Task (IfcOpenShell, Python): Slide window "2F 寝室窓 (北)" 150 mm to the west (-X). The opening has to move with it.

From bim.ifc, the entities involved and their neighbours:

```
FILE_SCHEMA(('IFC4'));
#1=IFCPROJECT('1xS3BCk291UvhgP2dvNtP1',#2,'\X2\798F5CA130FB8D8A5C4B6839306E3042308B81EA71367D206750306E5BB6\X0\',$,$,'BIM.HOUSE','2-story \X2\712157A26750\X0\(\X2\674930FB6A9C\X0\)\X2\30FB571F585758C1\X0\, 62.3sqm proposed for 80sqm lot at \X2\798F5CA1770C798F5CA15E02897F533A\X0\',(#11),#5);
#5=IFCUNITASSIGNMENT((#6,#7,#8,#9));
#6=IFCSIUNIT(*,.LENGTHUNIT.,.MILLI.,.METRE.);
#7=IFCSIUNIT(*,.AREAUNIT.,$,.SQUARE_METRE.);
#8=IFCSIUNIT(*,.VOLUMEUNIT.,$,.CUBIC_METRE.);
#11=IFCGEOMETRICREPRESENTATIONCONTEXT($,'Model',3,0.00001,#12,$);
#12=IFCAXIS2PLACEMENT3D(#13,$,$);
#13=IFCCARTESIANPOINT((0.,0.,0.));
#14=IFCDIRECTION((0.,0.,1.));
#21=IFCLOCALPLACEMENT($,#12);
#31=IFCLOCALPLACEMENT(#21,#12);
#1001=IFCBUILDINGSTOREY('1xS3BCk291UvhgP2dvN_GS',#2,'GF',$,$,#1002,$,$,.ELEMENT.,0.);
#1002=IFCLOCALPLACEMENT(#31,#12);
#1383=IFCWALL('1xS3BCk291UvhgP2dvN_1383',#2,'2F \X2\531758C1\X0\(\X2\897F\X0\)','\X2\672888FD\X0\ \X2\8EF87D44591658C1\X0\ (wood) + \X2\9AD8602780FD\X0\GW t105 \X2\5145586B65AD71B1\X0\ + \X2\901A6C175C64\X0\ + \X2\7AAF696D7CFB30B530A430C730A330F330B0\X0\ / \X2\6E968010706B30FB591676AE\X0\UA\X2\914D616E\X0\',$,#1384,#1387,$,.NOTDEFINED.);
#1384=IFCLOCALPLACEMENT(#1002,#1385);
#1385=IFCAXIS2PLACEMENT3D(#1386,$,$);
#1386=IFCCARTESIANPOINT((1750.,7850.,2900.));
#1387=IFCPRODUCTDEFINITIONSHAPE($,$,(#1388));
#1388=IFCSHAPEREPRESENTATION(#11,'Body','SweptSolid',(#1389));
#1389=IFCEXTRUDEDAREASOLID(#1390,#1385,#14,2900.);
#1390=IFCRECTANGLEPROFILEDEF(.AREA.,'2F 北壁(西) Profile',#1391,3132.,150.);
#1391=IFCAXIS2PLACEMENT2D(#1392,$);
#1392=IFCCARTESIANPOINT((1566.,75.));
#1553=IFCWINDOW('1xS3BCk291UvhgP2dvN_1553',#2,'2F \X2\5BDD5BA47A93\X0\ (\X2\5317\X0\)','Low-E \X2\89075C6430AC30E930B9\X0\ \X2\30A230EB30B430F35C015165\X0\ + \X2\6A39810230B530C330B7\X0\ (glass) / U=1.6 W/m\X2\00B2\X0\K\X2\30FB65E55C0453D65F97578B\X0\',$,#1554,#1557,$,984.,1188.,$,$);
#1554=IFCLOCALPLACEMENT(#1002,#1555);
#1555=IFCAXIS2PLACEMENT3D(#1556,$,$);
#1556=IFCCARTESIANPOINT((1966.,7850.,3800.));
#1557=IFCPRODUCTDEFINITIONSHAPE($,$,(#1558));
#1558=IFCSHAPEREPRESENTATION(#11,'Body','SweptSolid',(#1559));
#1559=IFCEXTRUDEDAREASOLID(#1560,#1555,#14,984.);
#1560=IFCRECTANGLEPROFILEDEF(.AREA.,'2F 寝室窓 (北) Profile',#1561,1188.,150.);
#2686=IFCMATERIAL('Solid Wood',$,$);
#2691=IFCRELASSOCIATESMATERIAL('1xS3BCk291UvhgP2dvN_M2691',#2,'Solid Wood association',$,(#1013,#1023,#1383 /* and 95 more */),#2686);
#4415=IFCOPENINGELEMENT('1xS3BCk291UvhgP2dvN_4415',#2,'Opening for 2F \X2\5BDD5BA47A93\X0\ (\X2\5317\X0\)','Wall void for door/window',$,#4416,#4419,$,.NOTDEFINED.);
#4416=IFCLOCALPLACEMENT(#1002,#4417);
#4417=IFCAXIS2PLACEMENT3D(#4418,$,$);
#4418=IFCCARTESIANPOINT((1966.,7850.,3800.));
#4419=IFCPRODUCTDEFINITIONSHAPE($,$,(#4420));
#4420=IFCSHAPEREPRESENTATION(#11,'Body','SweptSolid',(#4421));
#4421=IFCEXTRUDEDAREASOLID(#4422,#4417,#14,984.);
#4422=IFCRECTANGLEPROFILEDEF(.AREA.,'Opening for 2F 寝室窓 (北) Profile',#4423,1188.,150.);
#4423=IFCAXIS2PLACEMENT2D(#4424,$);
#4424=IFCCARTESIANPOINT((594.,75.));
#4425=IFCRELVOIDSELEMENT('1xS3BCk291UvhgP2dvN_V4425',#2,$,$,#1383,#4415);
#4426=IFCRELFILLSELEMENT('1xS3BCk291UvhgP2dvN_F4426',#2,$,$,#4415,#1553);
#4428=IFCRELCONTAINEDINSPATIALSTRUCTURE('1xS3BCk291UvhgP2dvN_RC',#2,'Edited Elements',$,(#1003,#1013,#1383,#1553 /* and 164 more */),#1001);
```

```python
import ifcopenshell
import ifcopenshell.api.geometry
import ifcopenshell.util.placement

model = ifcopenshell.open("bim.ifc")

window = model.by_id(1553)
opening = window.FillsVoids[0].RelatingOpeningElement
wall = opening.VoidsElements[0].RelatingBuildingElement

wall_matrix = ifcopenshell.util.placement.get_local_placement(wall.ObjectPlacement)
shift = wall_matrix[:3, 0] * -150.0
before = ifcopenshell.util.placement.get_local_placement(window.ObjectPlacement)[:3, 3].copy()

# The window is not placed relative to its opening, so move both.
for product in (opening, window):
    matrix = ifcopenshell.util.placement.get_local_placement(product.ObjectPlacement)
    matrix[:3, 3] += shift
    ifcopenshell.api.geometry.edit_object_placement(model, product=product, matrix=matrix, is_si=False)

after = ifcopenshell.util.placement.get_local_placement(window.ObjectPlacement)[:3, 3]
print("window moved by", (after - before).round(3) + 0.0)

model.write("bim_rev.ifc")
```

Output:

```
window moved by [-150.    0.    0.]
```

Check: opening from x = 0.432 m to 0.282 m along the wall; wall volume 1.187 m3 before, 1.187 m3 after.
